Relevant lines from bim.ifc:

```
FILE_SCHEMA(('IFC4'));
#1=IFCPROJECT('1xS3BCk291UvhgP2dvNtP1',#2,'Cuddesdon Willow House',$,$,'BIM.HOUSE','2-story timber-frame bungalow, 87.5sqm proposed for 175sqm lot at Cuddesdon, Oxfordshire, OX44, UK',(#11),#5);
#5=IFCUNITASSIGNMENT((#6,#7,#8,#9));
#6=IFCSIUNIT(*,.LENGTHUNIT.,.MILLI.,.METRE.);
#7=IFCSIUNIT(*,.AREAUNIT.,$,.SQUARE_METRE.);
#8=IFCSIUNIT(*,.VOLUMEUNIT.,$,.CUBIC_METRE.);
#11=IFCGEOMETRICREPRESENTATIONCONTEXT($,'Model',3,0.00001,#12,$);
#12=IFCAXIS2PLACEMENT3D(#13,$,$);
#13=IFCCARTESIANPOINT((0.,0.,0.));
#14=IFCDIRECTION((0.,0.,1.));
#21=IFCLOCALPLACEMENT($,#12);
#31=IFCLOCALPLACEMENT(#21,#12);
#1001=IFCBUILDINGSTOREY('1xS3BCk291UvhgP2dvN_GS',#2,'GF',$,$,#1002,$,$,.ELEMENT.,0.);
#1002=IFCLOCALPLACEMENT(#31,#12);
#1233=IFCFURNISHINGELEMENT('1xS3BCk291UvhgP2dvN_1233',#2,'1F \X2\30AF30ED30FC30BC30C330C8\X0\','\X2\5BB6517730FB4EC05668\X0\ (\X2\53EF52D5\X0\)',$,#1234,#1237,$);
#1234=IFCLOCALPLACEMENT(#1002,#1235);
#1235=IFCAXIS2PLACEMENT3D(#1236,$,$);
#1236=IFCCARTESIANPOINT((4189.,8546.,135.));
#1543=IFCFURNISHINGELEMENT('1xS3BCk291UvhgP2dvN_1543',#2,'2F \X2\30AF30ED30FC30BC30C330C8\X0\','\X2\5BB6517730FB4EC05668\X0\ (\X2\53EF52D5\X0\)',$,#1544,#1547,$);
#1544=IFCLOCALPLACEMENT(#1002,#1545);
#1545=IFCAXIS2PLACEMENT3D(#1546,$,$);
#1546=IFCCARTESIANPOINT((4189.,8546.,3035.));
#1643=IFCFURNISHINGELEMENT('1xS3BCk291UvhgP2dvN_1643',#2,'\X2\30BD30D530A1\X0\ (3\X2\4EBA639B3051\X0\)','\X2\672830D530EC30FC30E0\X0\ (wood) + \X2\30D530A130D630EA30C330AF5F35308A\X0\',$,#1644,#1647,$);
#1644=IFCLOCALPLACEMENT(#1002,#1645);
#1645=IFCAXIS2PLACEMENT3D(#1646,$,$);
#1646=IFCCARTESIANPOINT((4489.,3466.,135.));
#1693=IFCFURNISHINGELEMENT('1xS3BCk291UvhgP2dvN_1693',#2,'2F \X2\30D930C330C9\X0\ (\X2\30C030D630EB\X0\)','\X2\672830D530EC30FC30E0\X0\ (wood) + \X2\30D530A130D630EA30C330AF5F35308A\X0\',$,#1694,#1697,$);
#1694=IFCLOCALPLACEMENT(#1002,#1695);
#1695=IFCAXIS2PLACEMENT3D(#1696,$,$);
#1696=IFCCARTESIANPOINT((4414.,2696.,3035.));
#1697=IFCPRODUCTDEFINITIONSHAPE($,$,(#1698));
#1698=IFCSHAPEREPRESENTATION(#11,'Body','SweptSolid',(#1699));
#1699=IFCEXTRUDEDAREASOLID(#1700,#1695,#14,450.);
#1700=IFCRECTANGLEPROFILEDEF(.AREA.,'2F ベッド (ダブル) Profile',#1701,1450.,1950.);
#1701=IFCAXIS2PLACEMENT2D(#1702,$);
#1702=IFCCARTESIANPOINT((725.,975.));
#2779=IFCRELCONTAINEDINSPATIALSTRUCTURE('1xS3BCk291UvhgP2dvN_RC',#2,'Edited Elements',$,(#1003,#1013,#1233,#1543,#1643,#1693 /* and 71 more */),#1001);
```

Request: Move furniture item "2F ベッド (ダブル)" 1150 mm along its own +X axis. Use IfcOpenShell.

```python
import ifcopenshell
import ifcopenshell.api.geometry
import ifcopenshell.util.placement
import ifcopenshell.util.unit

model = ifcopenshell.open("bim.ifc")
unit_scale = ifcopenshell.util.unit.calculate_unit_scale(model)

item = model.by_guid("1xS3BCk291UvhgP2dvN_1693")
matrix = ifcopenshell.util.placement.get_local_placement(item.ObjectPlacement)
matrix[:3, 3] += matrix[:3, 0] * 1.15 / unit_scale
ifcopenshell.api.geometry.edit_object_placement(model, product=item, matrix=matrix, is_si=False)

print(ifcopenshell.util.placement.get_local_placement(item.ObjectPlacement).round(3) + 0.0)

model.write("bim_updated.ifc")
```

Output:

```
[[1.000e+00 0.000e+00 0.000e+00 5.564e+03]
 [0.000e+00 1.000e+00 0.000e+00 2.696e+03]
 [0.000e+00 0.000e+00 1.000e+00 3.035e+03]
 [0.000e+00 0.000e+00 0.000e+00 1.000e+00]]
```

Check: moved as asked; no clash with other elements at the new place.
